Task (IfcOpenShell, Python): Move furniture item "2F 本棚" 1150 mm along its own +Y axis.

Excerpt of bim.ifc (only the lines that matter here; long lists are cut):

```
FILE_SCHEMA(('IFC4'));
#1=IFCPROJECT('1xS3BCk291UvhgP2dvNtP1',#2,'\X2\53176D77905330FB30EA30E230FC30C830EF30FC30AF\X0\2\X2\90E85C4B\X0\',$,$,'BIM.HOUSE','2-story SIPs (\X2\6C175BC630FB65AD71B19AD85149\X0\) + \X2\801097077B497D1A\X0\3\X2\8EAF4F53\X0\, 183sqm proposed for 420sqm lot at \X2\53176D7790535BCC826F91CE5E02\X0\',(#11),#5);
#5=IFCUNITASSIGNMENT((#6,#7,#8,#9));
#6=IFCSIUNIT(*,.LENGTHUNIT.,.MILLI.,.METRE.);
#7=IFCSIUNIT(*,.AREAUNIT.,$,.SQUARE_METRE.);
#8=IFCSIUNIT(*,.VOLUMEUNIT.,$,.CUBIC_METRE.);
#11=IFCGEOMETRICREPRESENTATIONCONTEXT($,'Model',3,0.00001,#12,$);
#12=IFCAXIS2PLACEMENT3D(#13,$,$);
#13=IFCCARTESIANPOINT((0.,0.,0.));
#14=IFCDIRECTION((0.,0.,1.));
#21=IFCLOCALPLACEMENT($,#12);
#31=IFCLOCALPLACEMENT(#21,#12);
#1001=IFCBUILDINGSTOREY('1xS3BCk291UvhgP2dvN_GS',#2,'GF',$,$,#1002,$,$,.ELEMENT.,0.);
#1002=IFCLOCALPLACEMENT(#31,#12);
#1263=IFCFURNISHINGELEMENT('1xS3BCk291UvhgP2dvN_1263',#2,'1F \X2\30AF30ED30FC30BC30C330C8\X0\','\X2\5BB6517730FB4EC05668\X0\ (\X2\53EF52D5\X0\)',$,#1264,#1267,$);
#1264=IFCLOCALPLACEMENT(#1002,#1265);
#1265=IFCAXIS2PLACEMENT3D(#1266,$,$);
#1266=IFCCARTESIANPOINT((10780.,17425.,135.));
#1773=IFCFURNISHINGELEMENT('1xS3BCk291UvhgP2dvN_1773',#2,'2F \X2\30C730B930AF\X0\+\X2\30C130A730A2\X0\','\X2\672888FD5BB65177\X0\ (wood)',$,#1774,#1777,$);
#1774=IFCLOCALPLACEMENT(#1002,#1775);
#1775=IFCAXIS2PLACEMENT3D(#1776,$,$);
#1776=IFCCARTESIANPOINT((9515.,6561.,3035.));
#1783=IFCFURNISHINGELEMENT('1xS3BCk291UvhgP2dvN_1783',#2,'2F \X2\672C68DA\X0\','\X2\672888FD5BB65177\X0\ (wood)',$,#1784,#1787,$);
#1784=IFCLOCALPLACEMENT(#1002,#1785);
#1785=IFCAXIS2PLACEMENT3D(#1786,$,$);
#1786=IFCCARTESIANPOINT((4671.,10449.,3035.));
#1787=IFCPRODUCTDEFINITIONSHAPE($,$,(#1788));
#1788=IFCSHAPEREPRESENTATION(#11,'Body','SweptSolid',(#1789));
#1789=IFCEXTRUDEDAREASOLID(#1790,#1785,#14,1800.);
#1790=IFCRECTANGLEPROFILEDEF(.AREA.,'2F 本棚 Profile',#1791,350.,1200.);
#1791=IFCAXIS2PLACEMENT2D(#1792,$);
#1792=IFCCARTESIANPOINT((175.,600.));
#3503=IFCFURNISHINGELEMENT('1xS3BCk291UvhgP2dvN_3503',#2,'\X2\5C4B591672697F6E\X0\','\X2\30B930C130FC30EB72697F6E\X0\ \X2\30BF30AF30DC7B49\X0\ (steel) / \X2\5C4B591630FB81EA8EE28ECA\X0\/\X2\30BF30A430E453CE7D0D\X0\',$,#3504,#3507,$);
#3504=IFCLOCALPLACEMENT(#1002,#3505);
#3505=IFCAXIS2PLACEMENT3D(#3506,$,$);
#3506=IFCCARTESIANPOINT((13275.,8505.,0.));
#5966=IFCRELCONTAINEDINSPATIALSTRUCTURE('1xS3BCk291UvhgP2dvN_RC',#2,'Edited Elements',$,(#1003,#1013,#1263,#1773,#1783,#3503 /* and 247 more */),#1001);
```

```python
import ifcopenshell
import ifcopenshell.api.geometry
import ifcopenshell.util.placement

model = ifcopenshell.open("bim.ifc")

item = model.by_guid("1xS3BCk291UvhgP2dvN_1783")
matrix = ifcopenshell.util.placement.get_local_placement(item.ObjectPlacement)
matrix[:3, 3] += matrix[:3, 1] * 1150.0
ifcopenshell.api.geometry.edit_object_placement(model, product=item, matrix=matrix, is_si=False)

print(ifcopenshell.util.placement.get_local_placement(item.ObjectPlacement).round(3) + 0.0)

model.write("bim_updated.ifc")
```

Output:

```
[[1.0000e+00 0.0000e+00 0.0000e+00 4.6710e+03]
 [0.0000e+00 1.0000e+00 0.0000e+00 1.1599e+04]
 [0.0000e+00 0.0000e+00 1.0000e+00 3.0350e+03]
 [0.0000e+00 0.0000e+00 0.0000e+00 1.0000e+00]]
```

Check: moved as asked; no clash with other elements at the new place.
